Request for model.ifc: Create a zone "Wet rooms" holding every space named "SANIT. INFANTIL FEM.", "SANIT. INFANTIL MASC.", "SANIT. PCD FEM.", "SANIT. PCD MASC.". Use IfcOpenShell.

First a look at what the model holds.

```python
import ifcopenshell

model = ifcopenshell.open("model.ifc")
print(model.schema)
seen = {}
for space in model.by_type("IfcSpace"):
    seen[space.LongName] = seen.get(space.LongName, 0) + 1
for name, count in sorted(seen.items(), key=str):
    print(count, "x", name)
print("zones:", [z.Name for z in model.by_type("IfcZone")][:20])
```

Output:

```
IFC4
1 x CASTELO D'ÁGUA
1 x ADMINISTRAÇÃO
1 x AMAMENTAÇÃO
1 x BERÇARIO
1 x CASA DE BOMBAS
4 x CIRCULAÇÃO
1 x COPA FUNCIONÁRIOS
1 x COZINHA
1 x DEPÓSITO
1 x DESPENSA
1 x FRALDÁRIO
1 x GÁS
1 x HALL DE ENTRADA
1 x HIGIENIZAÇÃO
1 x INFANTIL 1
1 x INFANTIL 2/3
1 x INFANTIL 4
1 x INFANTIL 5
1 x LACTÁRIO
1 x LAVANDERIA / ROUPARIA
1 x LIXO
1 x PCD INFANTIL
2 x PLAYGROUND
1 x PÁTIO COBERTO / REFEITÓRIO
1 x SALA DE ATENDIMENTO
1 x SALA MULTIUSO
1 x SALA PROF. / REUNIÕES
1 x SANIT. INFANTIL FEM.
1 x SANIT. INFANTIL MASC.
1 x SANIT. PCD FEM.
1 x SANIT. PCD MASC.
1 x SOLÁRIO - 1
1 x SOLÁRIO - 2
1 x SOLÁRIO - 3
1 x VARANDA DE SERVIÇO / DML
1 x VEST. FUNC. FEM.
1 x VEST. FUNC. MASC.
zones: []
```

```python
import ifcopenshell
import ifcopenshell.api.group
import ifcopenshell.api.root

model = ifcopenshell.open("model.ifc")

names = {"SANIT. INFANTIL FEM.", "SANIT. INFANTIL MASC.", "SANIT. PCD FEM.", "SANIT. PCD MASC."}
spaces = [s for s in model.by_type("IfcSpace") if s.LongName in names]

zone = ifcopenshell.api.root.create_entity(model, ifc_class="IfcZone", name="Wet rooms")
ifcopenshell.api.group.assign_group(model, products=spaces, group=zone)
print(len(spaces), "spaces in", zone.Name)

model.write("model_edited.ifc")
```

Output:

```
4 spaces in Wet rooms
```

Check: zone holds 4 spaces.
